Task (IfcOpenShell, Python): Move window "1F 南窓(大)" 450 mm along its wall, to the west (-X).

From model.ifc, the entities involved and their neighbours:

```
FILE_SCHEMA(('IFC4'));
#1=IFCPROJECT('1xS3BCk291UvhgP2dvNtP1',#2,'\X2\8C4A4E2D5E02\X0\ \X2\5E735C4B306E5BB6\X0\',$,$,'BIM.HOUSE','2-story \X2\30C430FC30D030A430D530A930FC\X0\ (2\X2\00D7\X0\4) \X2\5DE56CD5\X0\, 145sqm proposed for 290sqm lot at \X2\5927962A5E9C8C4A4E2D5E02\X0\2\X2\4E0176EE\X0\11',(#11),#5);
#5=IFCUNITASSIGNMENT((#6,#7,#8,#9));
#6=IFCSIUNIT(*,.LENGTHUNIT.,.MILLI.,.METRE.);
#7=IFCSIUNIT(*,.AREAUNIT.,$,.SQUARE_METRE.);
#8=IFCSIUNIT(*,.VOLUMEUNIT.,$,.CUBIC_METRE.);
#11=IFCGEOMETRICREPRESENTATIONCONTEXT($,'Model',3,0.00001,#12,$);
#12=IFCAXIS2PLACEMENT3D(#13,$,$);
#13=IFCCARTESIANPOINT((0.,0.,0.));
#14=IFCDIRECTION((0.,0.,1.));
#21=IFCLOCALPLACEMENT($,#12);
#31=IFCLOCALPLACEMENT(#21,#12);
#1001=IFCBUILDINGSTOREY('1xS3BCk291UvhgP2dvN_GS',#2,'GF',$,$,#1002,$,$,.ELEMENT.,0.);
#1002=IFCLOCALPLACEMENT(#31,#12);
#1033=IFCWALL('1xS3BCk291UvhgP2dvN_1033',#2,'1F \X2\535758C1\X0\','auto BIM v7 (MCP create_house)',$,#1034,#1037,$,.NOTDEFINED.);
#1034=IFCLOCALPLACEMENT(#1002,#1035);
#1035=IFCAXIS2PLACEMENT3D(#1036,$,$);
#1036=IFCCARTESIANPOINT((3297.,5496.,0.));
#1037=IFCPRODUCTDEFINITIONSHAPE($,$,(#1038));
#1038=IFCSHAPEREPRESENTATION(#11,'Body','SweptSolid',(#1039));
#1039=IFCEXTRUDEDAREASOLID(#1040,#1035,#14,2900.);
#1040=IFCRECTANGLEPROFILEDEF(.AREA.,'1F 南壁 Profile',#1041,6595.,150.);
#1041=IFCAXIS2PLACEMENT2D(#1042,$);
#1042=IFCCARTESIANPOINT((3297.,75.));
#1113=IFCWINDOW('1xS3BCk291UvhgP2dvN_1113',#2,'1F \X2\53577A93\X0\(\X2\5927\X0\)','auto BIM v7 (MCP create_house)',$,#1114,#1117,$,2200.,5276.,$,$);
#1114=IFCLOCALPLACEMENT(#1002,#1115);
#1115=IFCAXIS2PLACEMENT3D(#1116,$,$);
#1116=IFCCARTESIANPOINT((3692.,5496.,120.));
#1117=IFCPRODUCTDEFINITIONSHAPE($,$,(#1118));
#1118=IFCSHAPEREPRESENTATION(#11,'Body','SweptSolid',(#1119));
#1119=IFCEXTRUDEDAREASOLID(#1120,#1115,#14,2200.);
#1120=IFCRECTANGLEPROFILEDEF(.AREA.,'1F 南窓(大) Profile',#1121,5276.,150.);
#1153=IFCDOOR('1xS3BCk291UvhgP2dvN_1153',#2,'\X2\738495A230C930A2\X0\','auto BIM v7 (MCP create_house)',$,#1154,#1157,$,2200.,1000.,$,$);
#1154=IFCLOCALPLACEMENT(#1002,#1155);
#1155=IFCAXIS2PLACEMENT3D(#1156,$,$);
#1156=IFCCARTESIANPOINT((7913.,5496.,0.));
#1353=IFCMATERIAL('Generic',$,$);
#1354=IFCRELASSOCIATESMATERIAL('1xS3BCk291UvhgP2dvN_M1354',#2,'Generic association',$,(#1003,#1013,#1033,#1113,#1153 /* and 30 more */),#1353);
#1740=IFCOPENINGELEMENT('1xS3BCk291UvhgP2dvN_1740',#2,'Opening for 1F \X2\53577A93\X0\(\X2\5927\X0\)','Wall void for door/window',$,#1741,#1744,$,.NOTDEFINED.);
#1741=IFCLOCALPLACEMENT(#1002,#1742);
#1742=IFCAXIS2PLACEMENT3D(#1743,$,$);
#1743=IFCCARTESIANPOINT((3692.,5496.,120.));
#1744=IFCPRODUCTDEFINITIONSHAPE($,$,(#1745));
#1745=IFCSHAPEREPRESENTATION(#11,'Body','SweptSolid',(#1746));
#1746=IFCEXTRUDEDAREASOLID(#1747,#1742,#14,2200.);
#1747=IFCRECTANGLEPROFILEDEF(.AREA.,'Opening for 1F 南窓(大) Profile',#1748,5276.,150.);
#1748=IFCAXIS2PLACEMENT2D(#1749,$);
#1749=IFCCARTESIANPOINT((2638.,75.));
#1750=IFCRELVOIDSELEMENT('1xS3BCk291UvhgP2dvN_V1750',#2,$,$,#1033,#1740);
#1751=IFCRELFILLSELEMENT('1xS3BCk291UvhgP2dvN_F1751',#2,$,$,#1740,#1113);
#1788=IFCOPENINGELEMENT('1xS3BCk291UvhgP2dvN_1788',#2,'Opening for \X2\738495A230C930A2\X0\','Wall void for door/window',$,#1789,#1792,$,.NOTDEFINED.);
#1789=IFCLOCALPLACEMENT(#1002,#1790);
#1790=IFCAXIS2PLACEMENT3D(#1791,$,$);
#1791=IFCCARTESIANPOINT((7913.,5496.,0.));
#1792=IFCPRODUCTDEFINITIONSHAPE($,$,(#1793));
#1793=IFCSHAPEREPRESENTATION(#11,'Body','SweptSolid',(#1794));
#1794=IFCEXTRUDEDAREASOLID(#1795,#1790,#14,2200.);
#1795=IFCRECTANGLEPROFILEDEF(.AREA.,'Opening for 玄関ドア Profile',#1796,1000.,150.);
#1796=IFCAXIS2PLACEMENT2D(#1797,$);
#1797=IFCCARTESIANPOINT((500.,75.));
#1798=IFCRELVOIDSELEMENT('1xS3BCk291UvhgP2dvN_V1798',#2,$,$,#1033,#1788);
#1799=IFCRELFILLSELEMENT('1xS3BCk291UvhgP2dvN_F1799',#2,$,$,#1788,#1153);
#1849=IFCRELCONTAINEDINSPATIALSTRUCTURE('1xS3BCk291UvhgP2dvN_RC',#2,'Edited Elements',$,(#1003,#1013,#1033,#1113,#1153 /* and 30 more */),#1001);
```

```python
import ifcopenshell
import ifcopenshell.api.geometry
import ifcopenshell.util.placement
import ifcopenshell.util.unit

model = ifcopenshell.open("model.ifc")
unit_scale = ifcopenshell.util.unit.calculate_unit_scale(model)

window = model.by_guid("1xS3BCk291UvhgP2dvN_1113")
opening = window.FillsVoids[0].RelatingOpeningElement
wall = opening.VoidsElements[0].RelatingBuildingElement

wall_matrix = ifcopenshell.util.placement.get_local_placement(wall.ObjectPlacement)
shift = wall_matrix[:3, 0] * -0.45 / unit_scale
before = ifcopenshell.util.placement.get_local_placement(window.ObjectPlacement)[:3, 3].copy()

# The window is not placed relative to its opening, so move both.
for product in (opening, window):
    matrix = ifcopenshell.util.placement.get_local_placement(product.ObjectPlacement)
    matrix[:3, 3] += shift
    ifcopenshell.api.geometry.edit_object_placement(model, product=product, matrix=matrix, is_si=False)

after = ifcopenshell.util.placement.get_local_placement(window.ObjectPlacement)[:3, 3]
print("window moved by", (after - before).round(3) + 0.0)

model.write("model_updated.ifc")
```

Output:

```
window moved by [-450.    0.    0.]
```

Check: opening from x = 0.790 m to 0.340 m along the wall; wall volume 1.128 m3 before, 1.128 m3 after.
